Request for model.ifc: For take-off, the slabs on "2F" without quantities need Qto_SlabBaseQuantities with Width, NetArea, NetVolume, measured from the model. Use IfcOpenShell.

First a look at what the model holds.

```python
import ifcopenshell
import ifcopenshell.util.element
import ifcopenshell.util.unit

model = ifcopenshell.open("model.ifc")
print(model.schema)
for unit_type in ("LENGTHUNIT", "AREAUNIT", "VOLUMEUNIT"):
    print(unit_type, ifcopenshell.util.unit.calculate_unit_scale(model, unit_type))
storey = next(s for s in model.by_type("IfcBuildingStorey") if s.Name == "2F")
slabs = [e for e in ifcopenshell.util.element.get_decomposition(storey) if e.is_a("IfcSlab")]
for e in sorted(slabs, key=lambda e: e.id()):
    print(e.id(), e.is_a(), e.Name, list(ifcopenshell.util.element.get_psets(e, qtos_only=True)), sep=" | ")
```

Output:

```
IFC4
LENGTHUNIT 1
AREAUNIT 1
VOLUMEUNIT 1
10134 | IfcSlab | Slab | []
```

```python
import ifcopenshell
import ifcopenshell.api.pset
import ifcopenshell.geom
import ifcopenshell.util.element
import ifcopenshell.util.shape
import ifcopenshell.util.unit

model = ifcopenshell.open("model.ifc")
unit_scale = ifcopenshell.util.unit.calculate_unit_scale(model)
area_scale = ifcopenshell.util.unit.calculate_unit_scale(model, "AREAUNIT")
volume_scale = ifcopenshell.util.unit.calculate_unit_scale(model, "VOLUMEUNIT")
settings = ifcopenshell.geom.settings()

storey = next(s for s in model.by_type("IfcBuildingStorey") if s.Name == "2F")
slabs = [e for e in ifcopenshell.util.element.get_decomposition(storey) if e.is_a("IfcSlab")]

for e in sorted(slabs, key=lambda e: e.id()):
    if ifcopenshell.util.element.get_psets(e, qtos_only=True, should_inherit=False):
        continue
    # Geometry comes back in metres, in the element's own axes.
    shape = ifcopenshell.geom.create_shape(settings, e)
    values = {
        "Width": ifcopenshell.util.shape.get_z(shape.geometry) / unit_scale,
        "NetArea": ifcopenshell.util.shape.get_footprint_area(shape.geometry) / area_scale,
        "NetVolume": ifcopenshell.util.shape.get_volume(shape.geometry) / volume_scale,
    }
    qto = ifcopenshell.api.pset.add_qto(model, product=e, name="Qto_SlabBaseQuantities")
    ifcopenshell.api.pset.edit_qto(model, qto=qto, properties=values)
    print(e.id(), {k: round(v, 3) for k, v in values.items()})

model.write("model_updated.ifc")
```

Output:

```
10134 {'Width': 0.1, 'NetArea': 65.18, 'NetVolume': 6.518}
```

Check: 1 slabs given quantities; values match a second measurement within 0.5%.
